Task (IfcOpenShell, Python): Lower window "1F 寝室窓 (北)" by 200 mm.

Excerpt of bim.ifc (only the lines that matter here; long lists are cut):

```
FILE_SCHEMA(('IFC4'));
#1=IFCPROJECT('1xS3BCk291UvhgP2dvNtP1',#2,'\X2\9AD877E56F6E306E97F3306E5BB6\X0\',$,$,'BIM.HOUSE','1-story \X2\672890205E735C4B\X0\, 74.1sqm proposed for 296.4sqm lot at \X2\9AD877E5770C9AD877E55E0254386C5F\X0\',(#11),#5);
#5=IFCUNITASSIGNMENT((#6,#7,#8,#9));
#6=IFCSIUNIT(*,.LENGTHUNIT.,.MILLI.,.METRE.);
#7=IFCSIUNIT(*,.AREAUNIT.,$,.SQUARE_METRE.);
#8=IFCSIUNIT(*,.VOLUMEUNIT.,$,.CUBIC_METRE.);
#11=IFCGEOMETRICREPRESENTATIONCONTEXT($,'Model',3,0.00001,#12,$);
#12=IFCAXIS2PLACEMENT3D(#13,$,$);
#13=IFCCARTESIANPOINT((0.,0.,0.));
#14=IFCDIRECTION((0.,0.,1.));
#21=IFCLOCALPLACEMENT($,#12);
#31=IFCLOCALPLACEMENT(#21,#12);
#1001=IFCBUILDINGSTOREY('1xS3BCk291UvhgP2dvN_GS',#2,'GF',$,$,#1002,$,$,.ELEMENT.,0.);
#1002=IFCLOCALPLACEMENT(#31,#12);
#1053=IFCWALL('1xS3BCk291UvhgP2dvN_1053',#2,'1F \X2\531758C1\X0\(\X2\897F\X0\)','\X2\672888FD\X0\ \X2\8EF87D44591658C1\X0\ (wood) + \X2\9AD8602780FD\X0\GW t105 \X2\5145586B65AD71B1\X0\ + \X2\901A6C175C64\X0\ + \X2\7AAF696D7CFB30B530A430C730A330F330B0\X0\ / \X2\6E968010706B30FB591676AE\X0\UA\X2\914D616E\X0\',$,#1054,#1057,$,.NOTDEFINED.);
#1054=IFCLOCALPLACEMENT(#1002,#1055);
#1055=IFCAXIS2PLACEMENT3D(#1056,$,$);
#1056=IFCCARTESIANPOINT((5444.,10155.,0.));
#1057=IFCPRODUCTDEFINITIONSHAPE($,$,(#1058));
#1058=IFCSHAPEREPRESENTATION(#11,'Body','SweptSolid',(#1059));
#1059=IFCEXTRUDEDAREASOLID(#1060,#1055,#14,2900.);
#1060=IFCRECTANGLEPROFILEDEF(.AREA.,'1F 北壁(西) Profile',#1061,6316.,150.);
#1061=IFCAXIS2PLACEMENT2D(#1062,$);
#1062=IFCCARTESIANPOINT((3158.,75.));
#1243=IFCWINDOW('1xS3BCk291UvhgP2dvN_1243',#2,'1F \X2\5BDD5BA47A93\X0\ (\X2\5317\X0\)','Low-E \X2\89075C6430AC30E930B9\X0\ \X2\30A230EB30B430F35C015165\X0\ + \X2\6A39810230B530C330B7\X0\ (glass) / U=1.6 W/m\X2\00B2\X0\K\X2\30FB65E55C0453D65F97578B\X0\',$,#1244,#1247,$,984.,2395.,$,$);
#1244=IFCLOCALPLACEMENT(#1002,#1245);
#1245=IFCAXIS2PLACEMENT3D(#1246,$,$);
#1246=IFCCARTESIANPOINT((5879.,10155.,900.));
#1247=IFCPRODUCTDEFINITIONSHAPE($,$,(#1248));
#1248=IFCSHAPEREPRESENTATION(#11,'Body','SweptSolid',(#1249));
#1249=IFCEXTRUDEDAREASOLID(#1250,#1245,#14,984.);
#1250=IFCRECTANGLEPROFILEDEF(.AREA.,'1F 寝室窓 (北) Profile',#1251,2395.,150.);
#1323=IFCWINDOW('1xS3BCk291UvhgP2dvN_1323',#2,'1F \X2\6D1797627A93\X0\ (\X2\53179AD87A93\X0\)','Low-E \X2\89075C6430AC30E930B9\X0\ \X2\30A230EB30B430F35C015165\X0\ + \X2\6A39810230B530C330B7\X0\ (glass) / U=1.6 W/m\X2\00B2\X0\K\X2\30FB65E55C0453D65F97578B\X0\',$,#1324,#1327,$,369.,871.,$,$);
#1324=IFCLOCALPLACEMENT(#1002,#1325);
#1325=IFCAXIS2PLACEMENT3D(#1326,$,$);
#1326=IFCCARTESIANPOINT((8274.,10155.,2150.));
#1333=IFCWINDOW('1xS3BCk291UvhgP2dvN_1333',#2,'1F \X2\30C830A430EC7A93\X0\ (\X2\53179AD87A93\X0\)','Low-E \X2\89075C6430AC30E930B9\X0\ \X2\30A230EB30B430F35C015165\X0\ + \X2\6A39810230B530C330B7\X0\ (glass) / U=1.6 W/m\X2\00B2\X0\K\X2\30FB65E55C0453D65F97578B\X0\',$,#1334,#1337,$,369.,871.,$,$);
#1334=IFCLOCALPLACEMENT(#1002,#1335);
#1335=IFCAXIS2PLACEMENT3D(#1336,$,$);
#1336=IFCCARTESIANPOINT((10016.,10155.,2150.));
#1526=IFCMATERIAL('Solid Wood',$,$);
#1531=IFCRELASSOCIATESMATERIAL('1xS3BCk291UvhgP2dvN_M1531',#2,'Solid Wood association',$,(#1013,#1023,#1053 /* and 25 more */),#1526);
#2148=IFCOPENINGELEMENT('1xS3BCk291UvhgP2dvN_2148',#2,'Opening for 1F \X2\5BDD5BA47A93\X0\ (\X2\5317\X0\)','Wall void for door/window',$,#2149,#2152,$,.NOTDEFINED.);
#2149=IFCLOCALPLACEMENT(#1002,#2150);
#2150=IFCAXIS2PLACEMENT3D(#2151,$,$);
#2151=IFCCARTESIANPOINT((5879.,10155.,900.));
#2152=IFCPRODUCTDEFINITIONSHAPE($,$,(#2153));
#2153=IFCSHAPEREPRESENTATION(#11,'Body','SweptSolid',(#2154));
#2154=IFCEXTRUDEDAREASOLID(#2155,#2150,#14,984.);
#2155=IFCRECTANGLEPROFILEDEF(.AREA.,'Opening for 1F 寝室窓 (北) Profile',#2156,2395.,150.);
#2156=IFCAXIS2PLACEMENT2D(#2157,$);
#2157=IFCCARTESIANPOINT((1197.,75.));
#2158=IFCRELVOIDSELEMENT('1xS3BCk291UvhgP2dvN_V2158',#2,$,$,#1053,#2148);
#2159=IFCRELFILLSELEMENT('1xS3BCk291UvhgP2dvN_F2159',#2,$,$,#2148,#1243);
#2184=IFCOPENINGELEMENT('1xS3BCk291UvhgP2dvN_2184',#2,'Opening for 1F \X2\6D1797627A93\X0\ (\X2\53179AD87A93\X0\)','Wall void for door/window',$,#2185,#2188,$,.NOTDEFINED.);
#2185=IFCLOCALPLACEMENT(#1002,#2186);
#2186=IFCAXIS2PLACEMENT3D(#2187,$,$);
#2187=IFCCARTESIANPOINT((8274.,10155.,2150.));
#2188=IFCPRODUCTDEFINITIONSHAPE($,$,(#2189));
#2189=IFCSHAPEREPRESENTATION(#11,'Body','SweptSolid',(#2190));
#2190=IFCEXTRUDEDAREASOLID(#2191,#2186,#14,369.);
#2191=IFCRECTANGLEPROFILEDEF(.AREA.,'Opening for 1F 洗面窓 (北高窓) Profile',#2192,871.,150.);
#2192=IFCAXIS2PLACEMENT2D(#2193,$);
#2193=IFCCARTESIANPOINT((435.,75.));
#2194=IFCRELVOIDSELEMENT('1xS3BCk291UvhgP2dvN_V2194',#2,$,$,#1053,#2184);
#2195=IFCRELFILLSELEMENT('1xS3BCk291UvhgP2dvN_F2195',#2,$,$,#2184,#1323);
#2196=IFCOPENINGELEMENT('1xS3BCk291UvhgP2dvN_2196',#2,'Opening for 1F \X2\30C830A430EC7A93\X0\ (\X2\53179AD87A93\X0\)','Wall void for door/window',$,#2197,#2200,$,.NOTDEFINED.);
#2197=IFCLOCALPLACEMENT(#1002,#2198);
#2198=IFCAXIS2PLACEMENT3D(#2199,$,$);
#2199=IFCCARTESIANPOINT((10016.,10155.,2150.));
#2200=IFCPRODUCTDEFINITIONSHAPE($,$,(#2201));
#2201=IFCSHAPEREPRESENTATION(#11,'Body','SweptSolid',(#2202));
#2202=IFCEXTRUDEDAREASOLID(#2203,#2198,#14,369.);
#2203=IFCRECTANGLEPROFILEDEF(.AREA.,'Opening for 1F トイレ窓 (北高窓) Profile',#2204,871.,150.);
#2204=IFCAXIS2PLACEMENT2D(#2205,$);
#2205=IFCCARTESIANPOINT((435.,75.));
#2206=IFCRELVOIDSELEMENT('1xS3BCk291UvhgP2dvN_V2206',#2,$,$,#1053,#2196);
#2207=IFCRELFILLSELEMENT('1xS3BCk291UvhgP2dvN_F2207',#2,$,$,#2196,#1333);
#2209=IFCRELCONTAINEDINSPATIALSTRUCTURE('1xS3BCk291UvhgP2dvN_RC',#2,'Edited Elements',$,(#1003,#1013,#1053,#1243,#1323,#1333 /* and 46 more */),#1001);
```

```python
import numpy as np
import ifcopenshell
import ifcopenshell.api.geometry
import ifcopenshell.util.placement
import ifcopenshell.util.unit

model = ifcopenshell.open("bim.ifc")
unit_scale = ifcopenshell.util.unit.calculate_unit_scale(model)

window = model.by_guid("1xS3BCk291UvhgP2dvN_1243")
opening = window.FillsVoids[0].RelatingOpeningElement
dz = -200.0

shift = np.array([0.0, 0.0, dz])
# The window is not placed relative to its opening, so move both.
for product in (opening, window):
    matrix = ifcopenshell.util.placement.get_local_placement(product.ObjectPlacement)
    matrix[:3, 3] += shift
    ifcopenshell.api.geometry.edit_object_placement(model, product=product, matrix=matrix, is_si=False)

print(f"moved by {dz * unit_scale:+.3f} m")

model.write("bim_rev.ifc")
```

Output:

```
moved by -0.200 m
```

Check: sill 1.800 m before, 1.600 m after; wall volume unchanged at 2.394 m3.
